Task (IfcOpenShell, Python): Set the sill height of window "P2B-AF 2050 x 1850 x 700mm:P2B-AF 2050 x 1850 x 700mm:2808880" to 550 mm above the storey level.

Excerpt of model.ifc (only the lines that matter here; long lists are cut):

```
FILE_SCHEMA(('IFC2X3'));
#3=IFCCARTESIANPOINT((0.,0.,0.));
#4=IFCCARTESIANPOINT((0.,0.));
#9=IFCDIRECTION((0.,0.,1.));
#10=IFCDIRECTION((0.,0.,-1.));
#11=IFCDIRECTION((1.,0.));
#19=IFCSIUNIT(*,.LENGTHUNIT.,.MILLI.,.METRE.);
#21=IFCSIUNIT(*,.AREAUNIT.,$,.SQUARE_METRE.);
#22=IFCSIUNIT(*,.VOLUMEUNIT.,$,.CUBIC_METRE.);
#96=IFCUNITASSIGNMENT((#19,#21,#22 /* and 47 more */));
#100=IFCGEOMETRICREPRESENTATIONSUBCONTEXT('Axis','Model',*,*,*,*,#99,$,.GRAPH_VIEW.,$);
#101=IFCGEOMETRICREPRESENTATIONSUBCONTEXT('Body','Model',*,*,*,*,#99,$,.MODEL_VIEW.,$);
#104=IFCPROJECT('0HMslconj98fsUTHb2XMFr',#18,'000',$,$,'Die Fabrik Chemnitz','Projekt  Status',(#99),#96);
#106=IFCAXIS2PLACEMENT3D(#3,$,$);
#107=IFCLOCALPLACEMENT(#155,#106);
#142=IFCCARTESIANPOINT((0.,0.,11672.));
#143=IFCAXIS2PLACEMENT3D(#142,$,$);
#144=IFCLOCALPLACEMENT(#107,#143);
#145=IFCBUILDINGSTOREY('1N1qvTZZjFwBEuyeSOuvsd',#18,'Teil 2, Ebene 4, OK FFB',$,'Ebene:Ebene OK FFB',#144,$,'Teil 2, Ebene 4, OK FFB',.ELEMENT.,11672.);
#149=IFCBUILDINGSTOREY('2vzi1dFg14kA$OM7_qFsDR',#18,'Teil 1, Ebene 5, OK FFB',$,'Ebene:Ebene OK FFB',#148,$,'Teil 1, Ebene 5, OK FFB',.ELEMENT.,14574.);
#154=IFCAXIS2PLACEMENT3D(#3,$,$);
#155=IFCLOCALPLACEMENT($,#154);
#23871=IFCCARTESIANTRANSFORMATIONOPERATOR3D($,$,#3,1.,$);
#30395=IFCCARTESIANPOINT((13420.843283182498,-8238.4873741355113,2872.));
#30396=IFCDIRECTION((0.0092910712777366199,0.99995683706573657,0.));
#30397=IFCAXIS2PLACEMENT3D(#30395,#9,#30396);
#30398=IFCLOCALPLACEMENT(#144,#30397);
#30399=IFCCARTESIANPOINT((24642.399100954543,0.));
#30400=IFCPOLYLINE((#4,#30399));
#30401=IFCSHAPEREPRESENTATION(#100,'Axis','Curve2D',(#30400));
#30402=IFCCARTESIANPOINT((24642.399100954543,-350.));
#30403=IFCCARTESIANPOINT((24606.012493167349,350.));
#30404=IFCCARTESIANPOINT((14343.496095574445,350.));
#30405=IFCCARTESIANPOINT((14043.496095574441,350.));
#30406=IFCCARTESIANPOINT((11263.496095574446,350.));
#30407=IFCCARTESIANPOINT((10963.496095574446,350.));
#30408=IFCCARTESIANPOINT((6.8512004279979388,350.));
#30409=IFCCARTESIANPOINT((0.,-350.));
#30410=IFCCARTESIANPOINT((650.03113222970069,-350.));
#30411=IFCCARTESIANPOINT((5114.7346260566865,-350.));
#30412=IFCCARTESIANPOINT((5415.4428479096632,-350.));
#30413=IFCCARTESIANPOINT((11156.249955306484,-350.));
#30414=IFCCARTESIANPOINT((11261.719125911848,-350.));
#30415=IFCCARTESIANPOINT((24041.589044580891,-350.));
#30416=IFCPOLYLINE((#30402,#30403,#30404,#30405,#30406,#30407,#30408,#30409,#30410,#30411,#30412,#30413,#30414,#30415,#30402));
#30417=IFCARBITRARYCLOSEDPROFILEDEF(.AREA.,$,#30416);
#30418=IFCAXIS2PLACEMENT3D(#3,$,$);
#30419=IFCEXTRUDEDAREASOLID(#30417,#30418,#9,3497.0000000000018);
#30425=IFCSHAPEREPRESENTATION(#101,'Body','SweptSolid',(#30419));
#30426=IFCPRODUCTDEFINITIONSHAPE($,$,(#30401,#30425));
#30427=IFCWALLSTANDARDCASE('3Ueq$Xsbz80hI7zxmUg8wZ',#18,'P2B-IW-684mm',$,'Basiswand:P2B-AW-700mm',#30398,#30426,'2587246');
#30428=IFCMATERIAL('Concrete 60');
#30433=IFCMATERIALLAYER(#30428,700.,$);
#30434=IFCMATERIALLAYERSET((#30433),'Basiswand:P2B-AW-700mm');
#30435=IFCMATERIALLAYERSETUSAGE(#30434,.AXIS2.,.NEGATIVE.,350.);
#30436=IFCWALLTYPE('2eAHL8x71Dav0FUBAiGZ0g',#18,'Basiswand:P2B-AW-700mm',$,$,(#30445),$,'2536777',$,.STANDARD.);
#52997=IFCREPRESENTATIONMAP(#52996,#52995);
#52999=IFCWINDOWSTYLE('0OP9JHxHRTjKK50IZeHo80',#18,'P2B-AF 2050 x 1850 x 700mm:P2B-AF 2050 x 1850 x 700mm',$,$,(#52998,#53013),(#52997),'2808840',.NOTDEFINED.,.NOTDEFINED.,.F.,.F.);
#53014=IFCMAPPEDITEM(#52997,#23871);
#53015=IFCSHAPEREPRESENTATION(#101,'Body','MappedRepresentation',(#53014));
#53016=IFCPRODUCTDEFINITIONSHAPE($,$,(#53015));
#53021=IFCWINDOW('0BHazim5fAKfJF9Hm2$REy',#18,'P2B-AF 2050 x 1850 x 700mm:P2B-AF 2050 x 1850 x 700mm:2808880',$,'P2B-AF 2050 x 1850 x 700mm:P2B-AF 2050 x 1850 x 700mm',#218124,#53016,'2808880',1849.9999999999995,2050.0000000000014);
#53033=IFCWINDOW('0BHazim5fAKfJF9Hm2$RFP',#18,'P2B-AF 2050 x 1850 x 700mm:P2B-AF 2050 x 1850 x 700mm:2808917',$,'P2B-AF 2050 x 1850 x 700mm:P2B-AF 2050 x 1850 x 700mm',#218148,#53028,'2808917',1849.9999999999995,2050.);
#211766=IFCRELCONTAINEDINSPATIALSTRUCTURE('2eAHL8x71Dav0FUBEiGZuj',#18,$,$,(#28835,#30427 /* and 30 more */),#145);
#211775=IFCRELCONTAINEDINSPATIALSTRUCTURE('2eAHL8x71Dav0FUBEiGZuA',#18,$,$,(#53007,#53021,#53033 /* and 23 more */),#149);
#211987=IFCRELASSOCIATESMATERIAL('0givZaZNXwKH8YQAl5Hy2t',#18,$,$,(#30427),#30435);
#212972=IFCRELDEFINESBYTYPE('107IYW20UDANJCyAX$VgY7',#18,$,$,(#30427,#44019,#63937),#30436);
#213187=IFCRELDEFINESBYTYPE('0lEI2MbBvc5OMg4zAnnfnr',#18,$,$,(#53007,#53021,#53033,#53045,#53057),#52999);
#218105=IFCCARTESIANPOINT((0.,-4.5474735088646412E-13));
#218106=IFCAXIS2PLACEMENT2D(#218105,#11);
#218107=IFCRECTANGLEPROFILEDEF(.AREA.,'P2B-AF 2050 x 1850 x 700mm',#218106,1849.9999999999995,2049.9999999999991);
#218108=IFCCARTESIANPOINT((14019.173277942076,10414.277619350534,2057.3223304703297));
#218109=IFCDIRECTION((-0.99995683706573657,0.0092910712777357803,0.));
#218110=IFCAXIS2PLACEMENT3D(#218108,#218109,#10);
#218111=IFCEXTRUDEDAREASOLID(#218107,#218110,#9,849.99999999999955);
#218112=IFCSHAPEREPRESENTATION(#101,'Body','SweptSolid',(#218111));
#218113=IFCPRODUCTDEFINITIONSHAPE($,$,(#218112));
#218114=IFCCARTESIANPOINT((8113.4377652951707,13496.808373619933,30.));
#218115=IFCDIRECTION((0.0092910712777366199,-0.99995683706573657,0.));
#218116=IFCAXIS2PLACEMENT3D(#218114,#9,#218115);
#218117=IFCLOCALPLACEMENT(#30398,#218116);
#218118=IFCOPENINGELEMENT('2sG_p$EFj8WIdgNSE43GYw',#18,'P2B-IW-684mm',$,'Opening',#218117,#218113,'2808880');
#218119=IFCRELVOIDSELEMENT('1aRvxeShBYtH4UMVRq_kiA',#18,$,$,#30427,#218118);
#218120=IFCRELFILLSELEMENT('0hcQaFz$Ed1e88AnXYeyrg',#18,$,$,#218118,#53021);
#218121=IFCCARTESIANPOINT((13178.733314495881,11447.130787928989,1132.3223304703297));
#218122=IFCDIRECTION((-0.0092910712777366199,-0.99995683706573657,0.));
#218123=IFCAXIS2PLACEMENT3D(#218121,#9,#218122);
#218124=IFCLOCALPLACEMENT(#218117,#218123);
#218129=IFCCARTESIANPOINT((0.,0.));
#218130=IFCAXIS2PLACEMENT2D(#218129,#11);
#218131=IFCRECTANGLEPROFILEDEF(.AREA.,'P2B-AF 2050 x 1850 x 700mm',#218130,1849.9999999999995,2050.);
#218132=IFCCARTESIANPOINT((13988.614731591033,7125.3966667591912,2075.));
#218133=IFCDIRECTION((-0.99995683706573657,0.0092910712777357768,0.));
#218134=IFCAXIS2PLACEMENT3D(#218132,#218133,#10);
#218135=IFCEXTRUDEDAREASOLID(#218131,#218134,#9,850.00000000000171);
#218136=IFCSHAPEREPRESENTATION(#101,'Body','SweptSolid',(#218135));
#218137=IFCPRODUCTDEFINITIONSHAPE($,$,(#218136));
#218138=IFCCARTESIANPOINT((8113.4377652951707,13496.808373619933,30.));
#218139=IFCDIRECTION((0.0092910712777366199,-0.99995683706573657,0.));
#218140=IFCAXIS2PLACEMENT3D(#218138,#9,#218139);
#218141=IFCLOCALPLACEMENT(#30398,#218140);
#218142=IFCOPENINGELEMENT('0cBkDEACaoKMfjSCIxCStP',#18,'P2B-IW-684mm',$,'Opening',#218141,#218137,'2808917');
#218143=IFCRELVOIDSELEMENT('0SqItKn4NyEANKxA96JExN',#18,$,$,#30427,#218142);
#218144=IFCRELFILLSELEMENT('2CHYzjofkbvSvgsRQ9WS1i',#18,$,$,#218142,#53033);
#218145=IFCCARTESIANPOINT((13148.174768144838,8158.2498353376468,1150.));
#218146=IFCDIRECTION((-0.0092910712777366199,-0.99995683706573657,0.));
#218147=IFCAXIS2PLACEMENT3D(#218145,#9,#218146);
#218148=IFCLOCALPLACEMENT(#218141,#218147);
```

```python
import numpy as np
import ifcopenshell
import ifcopenshell.api.geometry
import ifcopenshell.geom
import ifcopenshell.util.element
import ifcopenshell.util.placement
import ifcopenshell.util.shape
import ifcopenshell.util.unit

model = ifcopenshell.open("model.ifc")
unit_scale = ifcopenshell.util.unit.calculate_unit_scale(model)

window = model.by_guid("0BHazim5fAKfJF9Hm2$REy")
opening = window.FillsVoids[0].RelatingOpeningElement
storey = ifcopenshell.util.element.get_container(window, ifc_class="IfcBuildingStorey")
level = ifcopenshell.util.placement.get_local_placement(storey.ObjectPlacement)[2, 3]

# The opening's origin need not be at the sill, so measure its lowest point.
shape = ifcopenshell.geom.create_shape(ifcopenshell.geom.settings(), opening)
bottom = ifcopenshell.util.shape.get_shape_bottom_elevation(shape, shape.geometry) / unit_scale
dz = level + 0.55 / unit_scale - bottom

shift = np.array([0.0, 0.0, dz])
# The window is placed relative to its opening, so it follows when the opening moves.
matrix = ifcopenshell.util.placement.get_local_placement(opening.ObjectPlacement)
matrix[:3, 3] += shift
ifcopenshell.api.geometry.edit_object_placement(
    model, product=opening, matrix=matrix, is_si=False, should_transform_children=True
)

print(f"moved by {dz * unit_scale:+.3f} m")

model.write("model_edited.ifc")
```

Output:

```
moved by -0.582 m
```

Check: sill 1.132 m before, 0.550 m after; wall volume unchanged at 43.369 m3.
